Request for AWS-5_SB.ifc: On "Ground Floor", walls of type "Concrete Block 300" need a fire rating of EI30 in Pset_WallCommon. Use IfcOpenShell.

First a look at what the model holds.

```python
import ifcopenshell
import ifcopenshell.util.element

model = ifcopenshell.open("AWS-5_SB.ifc")
print(model.schema)
storey = next(s for s in model.by_type("IfcBuildingStorey") if s.Name == "Ground Floor")
walls = [e for e in ifcopenshell.util.element.get_decomposition(storey) if e.is_a("IfcWall")]
seen = {}
for e in walls:
    element_type = ifcopenshell.util.element.get_type(e)
    key = (element_type.Name if element_type != e and element_type else None, ifcopenshell.util.element.get_pset(e, "Pset_WallCommon", "FireRating"))
    seen[key] = seen.get(key, 0) + 1
for (name, value), count in sorted(seen.items(), key=str):
    print(count, "x", name, "|", value)
```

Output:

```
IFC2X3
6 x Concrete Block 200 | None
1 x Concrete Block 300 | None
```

```python
import ifcopenshell
import ifcopenshell.api.pset
import ifcopenshell.util.element

model = ifcopenshell.open("AWS-5_SB.ifc")

storey = next(s for s in model.by_type("IfcBuildingStorey") if s.Name == "Ground Floor")
walls = [e for e in ifcopenshell.util.element.get_decomposition(storey) if e.is_a("IfcWall")]

count = 0
for e in walls:
    element_type = ifcopenshell.util.element.get_type(e)
    if element_type in (None, e) or element_type.Name != "Concrete Block 300":
        continue
    # add_pset returns the element's existing set when there is one.
    pset = ifcopenshell.api.pset.add_pset(model, product=e, name="Pset_WallCommon")
    ifcopenshell.api.pset.edit_pset(model, pset=pset, properties={"FireRating": "EI30"})
    count += 1

print(count, "walls updated")

model.write("AWS-5_SB_edited.ifc")
```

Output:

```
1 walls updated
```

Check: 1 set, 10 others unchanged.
